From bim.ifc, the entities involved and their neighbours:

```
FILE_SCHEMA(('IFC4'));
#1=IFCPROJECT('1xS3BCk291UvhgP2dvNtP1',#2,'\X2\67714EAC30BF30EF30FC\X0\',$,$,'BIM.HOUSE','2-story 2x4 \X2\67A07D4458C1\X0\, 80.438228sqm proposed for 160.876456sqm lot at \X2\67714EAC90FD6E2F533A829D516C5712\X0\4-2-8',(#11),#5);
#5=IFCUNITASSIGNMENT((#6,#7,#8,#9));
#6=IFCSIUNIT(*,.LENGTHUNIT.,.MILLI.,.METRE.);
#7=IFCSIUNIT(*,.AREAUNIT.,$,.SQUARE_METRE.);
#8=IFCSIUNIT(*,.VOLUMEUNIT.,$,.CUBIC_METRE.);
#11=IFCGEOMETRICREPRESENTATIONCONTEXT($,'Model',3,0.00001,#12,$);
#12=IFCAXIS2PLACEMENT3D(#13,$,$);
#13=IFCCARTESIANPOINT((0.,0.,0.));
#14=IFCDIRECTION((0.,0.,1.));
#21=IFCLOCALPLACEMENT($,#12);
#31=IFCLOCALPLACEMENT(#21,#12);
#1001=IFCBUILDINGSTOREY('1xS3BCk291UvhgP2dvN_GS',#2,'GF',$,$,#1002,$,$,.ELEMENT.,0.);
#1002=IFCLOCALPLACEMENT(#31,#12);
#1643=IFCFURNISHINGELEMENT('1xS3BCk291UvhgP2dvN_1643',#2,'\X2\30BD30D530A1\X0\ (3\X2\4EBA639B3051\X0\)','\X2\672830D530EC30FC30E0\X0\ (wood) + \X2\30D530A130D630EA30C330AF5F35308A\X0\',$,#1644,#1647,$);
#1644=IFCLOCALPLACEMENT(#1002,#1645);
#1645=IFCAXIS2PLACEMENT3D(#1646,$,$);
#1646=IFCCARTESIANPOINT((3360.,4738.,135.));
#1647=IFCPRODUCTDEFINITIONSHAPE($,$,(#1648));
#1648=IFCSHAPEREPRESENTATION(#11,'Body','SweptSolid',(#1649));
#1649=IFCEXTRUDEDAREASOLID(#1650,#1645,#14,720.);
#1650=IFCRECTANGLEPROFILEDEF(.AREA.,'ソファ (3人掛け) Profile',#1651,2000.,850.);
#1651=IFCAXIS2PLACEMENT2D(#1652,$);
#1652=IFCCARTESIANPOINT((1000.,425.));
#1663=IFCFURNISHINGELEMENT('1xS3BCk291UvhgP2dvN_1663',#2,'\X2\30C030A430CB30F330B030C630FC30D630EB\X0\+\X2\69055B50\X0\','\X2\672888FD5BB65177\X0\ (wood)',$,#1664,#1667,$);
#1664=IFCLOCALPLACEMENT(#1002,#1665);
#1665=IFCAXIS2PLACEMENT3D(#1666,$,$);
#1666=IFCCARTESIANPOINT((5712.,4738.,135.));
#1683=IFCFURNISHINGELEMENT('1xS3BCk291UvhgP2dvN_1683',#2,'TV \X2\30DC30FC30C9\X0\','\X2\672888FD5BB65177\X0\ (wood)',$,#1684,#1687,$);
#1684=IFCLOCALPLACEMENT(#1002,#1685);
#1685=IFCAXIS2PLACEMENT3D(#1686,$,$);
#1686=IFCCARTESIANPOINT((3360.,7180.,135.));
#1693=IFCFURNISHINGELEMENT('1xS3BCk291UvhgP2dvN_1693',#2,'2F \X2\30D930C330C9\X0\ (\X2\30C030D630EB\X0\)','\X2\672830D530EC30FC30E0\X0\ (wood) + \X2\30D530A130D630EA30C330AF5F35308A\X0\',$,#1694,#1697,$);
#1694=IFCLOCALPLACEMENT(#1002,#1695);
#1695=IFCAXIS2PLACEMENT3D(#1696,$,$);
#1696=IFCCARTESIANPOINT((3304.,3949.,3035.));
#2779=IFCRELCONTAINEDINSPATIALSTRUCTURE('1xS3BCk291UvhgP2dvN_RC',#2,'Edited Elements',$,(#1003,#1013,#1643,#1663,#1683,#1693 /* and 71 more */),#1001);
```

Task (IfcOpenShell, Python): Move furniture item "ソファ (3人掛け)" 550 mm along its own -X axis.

```python
import ifcopenshell
import ifcopenshell.api.geometry
import ifcopenshell.util.placement
import ifcopenshell.util.unit

model = ifcopenshell.open("bim.ifc")
unit_scale = ifcopenshell.util.unit.calculate_unit_scale(model)

item = model.by_guid("1xS3BCk291UvhgP2dvN_1643")
matrix = ifcopenshell.util.placement.get_local_placement(item.ObjectPlacement)
matrix[:3, 3] -= matrix[:3, 0] * 0.55 / unit_scale
ifcopenshell.api.geometry.edit_object_placement(model, product=item, matrix=matrix, is_si=False)

print(ifcopenshell.util.placement.get_local_placement(item.ObjectPlacement).round(3) + 0.0)

model.write("bim_v2.ifc")
```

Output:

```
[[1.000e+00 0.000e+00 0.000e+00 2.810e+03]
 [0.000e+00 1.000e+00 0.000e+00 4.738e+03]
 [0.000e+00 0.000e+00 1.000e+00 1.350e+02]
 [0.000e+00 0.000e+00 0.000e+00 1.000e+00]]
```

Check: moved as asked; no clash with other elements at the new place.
